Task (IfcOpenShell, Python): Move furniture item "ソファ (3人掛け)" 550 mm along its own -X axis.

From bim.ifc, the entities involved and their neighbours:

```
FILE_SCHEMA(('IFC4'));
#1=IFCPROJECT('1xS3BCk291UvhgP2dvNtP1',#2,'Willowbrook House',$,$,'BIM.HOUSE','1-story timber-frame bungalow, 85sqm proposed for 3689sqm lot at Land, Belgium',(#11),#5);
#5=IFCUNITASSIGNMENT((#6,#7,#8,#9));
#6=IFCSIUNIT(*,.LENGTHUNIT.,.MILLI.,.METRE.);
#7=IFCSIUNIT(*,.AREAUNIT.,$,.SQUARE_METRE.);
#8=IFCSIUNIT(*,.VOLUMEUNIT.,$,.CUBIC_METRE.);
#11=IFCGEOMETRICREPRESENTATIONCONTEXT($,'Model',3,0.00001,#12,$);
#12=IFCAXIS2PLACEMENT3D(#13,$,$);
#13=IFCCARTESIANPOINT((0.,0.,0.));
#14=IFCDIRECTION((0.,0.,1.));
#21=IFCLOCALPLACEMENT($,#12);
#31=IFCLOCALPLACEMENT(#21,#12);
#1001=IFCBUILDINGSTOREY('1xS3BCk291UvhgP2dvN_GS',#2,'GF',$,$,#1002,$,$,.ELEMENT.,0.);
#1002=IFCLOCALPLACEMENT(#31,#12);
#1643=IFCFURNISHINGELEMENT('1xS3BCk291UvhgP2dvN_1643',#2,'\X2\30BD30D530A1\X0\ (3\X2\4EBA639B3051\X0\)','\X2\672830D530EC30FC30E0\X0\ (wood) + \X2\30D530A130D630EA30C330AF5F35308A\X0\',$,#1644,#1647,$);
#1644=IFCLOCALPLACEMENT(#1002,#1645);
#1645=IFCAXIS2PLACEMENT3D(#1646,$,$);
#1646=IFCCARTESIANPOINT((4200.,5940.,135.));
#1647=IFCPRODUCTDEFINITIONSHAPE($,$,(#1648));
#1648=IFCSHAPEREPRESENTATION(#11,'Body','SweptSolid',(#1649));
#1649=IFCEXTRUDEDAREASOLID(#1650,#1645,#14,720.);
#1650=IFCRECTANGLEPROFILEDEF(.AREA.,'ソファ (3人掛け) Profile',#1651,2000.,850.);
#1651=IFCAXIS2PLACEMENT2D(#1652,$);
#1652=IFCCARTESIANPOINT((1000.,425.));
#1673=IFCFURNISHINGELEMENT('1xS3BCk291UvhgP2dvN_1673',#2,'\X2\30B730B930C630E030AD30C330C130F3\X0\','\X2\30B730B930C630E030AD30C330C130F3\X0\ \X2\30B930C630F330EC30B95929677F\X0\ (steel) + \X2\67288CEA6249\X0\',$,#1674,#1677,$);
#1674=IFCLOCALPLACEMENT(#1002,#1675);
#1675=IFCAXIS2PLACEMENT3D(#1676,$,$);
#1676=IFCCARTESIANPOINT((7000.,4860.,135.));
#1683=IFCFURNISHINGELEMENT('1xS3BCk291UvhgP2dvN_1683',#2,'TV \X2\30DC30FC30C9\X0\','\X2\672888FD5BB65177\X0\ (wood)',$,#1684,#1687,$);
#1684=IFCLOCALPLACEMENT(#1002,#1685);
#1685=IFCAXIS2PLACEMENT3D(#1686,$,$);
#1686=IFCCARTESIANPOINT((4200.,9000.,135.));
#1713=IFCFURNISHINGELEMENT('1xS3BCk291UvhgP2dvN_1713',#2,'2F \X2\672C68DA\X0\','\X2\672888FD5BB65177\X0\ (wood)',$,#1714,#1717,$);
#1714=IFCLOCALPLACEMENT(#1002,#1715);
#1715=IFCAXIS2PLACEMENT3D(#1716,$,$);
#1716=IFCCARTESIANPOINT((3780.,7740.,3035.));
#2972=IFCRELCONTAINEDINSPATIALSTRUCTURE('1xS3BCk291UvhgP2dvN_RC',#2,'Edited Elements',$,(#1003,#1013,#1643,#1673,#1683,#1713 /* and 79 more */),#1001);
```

```python
import ifcopenshell
import ifcopenshell.api.geometry
import ifcopenshell.util.placement
import ifcopenshell.util.unit

model = ifcopenshell.open("bim.ifc")
unit_scale = ifcopenshell.util.unit.calculate_unit_scale(model)

item = model.by_id(1643)
matrix = ifcopenshell.util.placement.get_local_placement(item.ObjectPlacement)
matrix[:3, 3] -= matrix[:3, 0] * 0.55 / unit_scale
ifcopenshell.api.geometry.edit_object_placement(model, product=item, matrix=matrix, is_si=False)

print(ifcopenshell.util.placement.get_local_placement(item.ObjectPlacement).round(3) + 0.0)

model.write("bim_v2.ifc")
```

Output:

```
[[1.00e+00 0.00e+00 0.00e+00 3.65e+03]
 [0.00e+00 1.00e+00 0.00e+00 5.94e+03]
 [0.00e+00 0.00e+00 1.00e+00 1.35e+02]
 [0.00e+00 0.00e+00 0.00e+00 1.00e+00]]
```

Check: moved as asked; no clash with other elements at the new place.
